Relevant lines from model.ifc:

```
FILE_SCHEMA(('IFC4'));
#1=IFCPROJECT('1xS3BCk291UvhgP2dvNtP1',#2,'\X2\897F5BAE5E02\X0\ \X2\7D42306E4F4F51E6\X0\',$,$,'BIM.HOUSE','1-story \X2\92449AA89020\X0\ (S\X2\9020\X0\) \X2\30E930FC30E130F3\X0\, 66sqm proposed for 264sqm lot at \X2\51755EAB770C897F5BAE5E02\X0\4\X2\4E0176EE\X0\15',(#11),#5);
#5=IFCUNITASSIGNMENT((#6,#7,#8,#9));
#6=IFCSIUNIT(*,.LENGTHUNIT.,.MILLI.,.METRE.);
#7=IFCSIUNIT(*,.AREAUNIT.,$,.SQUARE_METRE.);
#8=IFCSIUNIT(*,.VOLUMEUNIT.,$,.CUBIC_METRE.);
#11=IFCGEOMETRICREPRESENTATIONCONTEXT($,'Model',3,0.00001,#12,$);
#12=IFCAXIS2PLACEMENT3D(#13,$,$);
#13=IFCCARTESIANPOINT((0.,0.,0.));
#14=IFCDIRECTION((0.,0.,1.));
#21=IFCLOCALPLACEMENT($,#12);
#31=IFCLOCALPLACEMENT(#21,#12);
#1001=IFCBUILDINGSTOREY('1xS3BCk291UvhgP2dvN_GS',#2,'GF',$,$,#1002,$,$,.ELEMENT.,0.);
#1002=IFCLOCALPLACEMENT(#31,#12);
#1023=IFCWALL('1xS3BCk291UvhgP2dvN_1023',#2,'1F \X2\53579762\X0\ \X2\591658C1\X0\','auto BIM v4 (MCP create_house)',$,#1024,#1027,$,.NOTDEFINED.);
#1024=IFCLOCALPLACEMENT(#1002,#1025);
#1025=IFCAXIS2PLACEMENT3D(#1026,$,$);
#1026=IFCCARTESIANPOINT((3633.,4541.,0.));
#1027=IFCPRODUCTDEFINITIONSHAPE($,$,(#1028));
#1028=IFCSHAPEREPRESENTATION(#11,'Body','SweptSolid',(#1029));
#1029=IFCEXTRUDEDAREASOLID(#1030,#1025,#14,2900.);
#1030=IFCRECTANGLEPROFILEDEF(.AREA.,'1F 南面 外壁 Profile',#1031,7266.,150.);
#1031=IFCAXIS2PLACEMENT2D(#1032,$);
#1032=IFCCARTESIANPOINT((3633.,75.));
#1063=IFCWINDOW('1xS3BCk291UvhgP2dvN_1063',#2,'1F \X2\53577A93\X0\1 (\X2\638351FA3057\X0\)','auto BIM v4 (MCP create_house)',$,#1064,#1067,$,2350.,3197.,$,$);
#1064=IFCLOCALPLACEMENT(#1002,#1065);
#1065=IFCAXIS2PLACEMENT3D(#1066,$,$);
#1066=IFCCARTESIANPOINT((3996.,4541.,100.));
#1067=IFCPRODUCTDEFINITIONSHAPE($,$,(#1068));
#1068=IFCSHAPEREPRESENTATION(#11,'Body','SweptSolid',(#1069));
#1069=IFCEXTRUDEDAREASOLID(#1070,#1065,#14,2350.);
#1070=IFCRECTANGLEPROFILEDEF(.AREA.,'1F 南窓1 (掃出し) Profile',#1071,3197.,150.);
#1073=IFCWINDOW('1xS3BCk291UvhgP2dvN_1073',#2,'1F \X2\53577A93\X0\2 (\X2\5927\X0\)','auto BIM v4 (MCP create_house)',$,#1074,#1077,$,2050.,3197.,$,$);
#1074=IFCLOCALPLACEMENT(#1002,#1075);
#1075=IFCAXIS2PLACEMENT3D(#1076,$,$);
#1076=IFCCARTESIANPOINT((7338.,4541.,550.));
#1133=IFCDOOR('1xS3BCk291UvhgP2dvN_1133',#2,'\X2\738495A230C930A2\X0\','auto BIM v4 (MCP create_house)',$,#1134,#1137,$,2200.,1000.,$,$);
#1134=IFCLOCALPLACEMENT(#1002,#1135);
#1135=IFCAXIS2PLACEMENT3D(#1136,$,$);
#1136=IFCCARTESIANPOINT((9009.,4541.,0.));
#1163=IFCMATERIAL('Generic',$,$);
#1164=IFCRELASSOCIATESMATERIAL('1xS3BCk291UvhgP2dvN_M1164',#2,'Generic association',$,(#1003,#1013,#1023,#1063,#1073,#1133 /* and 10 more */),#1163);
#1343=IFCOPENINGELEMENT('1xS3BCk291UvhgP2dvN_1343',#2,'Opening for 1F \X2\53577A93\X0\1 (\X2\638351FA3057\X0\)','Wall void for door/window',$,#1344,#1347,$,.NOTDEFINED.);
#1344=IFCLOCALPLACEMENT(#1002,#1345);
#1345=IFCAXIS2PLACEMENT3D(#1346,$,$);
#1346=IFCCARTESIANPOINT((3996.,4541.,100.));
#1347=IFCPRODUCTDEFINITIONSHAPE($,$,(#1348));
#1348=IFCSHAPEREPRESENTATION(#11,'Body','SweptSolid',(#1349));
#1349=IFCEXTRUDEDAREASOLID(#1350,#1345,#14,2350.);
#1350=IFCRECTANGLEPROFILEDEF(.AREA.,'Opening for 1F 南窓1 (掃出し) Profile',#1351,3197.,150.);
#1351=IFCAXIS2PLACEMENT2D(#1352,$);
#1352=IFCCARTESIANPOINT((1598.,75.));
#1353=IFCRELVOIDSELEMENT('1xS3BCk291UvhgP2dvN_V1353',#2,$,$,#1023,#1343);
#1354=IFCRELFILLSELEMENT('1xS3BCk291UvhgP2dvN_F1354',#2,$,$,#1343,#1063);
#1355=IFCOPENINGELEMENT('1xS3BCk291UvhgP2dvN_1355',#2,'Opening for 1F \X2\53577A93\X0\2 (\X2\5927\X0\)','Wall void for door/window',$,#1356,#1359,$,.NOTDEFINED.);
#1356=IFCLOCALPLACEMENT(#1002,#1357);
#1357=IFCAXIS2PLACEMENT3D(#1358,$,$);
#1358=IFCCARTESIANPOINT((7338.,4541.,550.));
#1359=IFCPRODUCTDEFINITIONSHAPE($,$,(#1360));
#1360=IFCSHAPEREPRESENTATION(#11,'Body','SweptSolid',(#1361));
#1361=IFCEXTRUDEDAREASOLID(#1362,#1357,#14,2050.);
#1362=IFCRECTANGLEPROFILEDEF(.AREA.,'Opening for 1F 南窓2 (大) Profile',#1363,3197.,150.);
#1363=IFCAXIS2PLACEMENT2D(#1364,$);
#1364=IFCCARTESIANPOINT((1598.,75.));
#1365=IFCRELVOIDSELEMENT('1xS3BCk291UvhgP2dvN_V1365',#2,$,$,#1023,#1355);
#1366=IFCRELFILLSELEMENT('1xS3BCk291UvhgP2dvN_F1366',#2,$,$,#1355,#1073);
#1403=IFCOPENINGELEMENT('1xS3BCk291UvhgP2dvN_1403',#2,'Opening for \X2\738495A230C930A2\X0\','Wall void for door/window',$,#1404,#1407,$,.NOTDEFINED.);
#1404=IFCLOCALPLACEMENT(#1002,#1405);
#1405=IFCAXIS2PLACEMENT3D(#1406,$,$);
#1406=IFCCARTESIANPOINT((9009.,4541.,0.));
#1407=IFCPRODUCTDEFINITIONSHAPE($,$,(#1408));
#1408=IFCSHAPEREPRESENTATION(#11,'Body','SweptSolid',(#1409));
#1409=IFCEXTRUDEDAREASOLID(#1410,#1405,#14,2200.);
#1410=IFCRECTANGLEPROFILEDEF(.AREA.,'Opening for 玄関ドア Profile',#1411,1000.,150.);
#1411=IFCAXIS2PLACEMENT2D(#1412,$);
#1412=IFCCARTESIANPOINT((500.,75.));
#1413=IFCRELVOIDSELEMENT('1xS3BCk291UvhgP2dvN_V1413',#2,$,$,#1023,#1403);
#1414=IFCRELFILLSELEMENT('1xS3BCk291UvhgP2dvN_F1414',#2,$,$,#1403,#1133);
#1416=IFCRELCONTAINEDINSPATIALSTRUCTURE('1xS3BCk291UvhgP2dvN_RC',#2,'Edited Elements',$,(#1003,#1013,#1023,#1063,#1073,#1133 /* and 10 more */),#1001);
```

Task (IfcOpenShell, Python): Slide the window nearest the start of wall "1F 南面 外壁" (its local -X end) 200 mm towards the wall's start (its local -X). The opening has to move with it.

```python
import ifcopenshell
import ifcopenshell.api.geometry
import ifcopenshell.util.placement
import ifcopenshell.util.unit

model = ifcopenshell.open("model.ifc")
unit_scale = ifcopenshell.util.unit.calculate_unit_scale(model)

window = model.by_guid("1xS3BCk291UvhgP2dvN_1063")
opening = window.FillsVoids[0].RelatingOpeningElement
wall = opening.VoidsElements[0].RelatingBuildingElement

wall_matrix = ifcopenshell.util.placement.get_local_placement(wall.ObjectPlacement)
shift = wall_matrix[:3, 0] * -0.2 / unit_scale
before = ifcopenshell.util.placement.get_local_placement(window.ObjectPlacement)[:3, 3].copy()

# The window is not placed relative to its opening, so move both.
for product in (opening, window):
    matrix = ifcopenshell.util.placement.get_local_placement(product.ObjectPlacement)
    matrix[:3, 3] += shift
    ifcopenshell.api.geometry.edit_object_placement(model, product=product, matrix=matrix, is_si=False)

after = ifcopenshell.util.placement.get_local_placement(window.ObjectPlacement)[:3, 3]
print("window moved by", (after - before).round(3) + 0.0)

model.write("model_v2.ifc")
```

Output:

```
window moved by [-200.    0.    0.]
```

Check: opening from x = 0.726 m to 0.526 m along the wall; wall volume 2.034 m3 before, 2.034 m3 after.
